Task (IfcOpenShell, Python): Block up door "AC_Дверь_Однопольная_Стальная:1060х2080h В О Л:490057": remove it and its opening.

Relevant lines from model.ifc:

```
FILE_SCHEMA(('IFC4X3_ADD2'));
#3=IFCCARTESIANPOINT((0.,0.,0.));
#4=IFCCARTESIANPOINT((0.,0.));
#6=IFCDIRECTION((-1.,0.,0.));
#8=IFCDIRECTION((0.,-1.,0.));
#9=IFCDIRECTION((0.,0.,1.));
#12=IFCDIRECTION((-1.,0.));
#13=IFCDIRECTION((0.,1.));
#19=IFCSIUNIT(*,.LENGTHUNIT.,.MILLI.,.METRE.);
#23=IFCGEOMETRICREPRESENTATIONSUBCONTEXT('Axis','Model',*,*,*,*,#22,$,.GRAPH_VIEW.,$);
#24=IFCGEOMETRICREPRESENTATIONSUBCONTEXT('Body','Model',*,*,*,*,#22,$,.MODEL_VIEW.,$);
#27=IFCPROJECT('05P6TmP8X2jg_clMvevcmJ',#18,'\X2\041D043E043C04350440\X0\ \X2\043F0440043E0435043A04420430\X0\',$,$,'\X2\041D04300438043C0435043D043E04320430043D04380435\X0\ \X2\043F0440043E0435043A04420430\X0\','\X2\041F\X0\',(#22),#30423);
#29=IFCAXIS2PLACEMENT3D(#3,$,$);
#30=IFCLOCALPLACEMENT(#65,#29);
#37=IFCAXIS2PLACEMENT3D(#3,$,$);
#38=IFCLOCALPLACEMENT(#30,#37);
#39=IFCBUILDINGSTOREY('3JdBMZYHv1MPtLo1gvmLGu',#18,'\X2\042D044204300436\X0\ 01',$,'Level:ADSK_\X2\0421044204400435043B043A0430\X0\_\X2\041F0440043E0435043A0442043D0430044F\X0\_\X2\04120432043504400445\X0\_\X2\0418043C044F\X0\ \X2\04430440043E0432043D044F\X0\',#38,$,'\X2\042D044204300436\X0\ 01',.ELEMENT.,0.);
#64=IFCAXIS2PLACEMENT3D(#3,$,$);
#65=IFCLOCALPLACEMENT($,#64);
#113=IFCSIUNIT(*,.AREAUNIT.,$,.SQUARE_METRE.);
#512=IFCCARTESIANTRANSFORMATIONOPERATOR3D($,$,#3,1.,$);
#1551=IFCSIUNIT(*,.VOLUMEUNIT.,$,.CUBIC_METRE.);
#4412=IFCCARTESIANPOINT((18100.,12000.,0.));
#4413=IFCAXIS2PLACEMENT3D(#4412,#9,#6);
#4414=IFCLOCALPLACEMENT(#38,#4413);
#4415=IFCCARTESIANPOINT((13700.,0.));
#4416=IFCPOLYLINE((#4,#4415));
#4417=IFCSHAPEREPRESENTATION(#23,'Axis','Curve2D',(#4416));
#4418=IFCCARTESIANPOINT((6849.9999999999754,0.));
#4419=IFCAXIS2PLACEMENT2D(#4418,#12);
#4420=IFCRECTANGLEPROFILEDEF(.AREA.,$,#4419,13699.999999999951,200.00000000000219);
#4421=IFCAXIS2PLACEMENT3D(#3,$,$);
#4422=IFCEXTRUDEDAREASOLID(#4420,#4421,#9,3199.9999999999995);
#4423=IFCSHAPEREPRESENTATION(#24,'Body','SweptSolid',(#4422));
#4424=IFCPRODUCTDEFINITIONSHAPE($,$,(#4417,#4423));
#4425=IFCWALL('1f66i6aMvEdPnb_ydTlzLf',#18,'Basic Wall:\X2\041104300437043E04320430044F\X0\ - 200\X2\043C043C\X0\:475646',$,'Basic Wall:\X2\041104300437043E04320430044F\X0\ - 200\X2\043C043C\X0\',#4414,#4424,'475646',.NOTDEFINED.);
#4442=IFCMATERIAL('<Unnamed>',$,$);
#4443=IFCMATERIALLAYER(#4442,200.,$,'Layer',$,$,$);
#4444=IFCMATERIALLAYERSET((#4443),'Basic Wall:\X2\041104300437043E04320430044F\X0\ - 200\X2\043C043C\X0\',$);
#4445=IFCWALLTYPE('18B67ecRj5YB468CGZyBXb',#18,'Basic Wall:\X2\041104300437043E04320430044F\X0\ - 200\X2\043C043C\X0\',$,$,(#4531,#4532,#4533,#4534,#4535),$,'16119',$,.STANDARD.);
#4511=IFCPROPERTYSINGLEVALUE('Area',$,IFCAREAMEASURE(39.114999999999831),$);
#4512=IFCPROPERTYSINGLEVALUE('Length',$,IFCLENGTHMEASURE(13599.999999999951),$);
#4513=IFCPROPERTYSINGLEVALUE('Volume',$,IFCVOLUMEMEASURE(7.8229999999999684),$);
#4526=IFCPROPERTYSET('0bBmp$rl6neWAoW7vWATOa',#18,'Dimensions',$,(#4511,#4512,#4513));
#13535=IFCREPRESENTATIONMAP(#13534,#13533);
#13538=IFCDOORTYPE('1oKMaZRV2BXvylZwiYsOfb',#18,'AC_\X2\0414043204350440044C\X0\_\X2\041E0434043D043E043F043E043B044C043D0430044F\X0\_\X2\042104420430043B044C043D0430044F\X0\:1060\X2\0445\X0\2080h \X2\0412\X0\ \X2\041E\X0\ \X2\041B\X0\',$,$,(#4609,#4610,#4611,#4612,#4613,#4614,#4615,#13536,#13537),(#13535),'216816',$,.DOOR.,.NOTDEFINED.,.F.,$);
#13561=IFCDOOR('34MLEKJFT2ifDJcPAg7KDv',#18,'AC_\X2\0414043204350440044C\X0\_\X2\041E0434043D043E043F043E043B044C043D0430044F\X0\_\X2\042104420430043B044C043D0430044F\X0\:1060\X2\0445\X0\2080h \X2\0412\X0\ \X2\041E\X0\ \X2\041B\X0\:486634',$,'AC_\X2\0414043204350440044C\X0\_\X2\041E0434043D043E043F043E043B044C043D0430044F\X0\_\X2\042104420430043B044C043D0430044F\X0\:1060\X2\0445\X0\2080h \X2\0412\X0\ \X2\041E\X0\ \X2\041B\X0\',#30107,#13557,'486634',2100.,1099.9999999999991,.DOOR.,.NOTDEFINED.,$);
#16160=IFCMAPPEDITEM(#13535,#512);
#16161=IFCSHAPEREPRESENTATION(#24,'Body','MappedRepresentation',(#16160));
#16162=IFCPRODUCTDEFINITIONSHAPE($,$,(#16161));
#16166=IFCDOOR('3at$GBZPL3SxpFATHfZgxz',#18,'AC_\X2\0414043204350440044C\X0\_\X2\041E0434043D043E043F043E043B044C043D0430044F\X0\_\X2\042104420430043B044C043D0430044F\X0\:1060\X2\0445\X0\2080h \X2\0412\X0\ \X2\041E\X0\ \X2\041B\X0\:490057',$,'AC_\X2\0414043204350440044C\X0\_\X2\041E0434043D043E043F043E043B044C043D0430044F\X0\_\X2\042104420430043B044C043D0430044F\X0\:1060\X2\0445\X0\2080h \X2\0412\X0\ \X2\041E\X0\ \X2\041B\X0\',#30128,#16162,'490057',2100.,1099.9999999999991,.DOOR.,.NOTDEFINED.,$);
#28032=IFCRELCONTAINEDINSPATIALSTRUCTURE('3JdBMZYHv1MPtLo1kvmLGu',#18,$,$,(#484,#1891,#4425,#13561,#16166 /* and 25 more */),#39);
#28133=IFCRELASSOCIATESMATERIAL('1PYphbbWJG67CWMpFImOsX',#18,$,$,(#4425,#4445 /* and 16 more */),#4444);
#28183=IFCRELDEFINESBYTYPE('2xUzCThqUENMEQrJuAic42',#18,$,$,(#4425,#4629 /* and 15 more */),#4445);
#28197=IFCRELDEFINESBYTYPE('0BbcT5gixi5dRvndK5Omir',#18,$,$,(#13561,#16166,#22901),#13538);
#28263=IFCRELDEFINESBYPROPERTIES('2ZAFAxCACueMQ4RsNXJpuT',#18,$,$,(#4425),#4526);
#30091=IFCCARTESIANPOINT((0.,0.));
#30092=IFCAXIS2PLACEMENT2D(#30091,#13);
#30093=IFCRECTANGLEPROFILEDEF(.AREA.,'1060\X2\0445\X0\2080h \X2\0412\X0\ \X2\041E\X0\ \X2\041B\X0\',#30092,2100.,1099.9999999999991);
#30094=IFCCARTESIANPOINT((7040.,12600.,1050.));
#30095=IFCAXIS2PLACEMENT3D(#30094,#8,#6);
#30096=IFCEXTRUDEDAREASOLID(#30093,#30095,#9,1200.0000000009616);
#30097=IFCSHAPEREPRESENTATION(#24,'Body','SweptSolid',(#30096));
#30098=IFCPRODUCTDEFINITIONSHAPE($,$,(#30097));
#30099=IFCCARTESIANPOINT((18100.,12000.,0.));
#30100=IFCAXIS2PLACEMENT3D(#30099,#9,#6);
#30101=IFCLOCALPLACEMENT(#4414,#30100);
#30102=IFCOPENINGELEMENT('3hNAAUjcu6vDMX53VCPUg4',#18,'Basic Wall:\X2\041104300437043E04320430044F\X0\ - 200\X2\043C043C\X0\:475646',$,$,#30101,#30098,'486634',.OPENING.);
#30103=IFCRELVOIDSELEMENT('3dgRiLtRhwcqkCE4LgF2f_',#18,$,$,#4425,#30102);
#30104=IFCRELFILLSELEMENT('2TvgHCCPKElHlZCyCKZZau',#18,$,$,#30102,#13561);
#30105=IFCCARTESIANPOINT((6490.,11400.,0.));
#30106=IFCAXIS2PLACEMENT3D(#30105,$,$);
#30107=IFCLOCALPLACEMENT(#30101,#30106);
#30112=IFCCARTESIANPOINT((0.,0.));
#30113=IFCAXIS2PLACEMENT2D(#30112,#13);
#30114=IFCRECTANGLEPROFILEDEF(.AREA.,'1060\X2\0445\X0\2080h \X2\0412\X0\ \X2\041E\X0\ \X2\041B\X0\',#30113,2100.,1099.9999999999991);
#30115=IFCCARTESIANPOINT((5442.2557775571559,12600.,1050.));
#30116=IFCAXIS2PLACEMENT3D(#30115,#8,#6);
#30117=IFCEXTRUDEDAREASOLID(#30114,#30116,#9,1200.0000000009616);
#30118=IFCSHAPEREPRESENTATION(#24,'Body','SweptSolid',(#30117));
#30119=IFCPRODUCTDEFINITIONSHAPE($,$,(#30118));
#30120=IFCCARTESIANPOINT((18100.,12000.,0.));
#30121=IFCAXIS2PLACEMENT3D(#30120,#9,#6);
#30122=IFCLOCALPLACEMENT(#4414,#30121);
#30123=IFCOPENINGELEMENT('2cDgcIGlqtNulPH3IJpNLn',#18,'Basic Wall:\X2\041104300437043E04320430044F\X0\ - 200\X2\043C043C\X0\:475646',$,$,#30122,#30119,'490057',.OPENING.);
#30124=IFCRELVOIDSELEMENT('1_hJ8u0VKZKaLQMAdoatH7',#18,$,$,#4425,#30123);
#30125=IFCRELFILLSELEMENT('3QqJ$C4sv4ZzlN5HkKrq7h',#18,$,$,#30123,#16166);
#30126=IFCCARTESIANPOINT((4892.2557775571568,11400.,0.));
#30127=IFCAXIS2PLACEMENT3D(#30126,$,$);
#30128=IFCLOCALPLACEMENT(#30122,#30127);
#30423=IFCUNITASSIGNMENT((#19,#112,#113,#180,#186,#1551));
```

```python
import ifcopenshell
import ifcopenshell.api.feature
import ifcopenshell.api.pset
import ifcopenshell.api.root
import ifcopenshell.geom
import ifcopenshell.util.element
import ifcopenshell.util.shape
import ifcopenshell.util.unit

model = ifcopenshell.open("model.ifc")
area_scale = ifcopenshell.util.unit.calculate_unit_scale(model, "AREAUNIT")
volume_scale = ifcopenshell.util.unit.calculate_unit_scale(model, "VOLUMEUNIT")
settings = ifcopenshell.geom.settings()


def volume(element):
    """Net volume in cubic metres, openings subtracted."""
    shape = ifcopenshell.geom.create_shape(settings, element)
    return ifcopenshell.util.shape.get_volume(shape.geometry)


door = model.by_id(16166)
opening = door.FillsVoids[0].RelatingOpeningElement
wall = opening.VoidsElements[0].RelatingBuildingElement
before = volume(wall)

ifcopenshell.api.root.remove_product(model, product=door)
ifcopenshell.api.feature.remove_feature(model, feature=opening)

after = volume(wall)
thickness = 0.2  # wall thickness in metres

# Update the wall's stored quantities.
pset = model.by_id(ifcopenshell.util.element.get_pset(wall, "Dimensions", should_inherit=False)["id"])
ifcopenshell.api.pset.edit_pset(model, pset=pset, properties={
    "Area": model.create_entity("IfcAreaMeasure", after / thickness / area_scale),
    "Volume": model.create_entity("IfcVolumeMeasure", after / volume_scale),
})

print(f"wall volume {before:.3f} -> {after:.3f} m3")

model.write("model-out.ifc")
```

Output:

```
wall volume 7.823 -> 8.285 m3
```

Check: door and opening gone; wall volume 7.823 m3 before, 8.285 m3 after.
